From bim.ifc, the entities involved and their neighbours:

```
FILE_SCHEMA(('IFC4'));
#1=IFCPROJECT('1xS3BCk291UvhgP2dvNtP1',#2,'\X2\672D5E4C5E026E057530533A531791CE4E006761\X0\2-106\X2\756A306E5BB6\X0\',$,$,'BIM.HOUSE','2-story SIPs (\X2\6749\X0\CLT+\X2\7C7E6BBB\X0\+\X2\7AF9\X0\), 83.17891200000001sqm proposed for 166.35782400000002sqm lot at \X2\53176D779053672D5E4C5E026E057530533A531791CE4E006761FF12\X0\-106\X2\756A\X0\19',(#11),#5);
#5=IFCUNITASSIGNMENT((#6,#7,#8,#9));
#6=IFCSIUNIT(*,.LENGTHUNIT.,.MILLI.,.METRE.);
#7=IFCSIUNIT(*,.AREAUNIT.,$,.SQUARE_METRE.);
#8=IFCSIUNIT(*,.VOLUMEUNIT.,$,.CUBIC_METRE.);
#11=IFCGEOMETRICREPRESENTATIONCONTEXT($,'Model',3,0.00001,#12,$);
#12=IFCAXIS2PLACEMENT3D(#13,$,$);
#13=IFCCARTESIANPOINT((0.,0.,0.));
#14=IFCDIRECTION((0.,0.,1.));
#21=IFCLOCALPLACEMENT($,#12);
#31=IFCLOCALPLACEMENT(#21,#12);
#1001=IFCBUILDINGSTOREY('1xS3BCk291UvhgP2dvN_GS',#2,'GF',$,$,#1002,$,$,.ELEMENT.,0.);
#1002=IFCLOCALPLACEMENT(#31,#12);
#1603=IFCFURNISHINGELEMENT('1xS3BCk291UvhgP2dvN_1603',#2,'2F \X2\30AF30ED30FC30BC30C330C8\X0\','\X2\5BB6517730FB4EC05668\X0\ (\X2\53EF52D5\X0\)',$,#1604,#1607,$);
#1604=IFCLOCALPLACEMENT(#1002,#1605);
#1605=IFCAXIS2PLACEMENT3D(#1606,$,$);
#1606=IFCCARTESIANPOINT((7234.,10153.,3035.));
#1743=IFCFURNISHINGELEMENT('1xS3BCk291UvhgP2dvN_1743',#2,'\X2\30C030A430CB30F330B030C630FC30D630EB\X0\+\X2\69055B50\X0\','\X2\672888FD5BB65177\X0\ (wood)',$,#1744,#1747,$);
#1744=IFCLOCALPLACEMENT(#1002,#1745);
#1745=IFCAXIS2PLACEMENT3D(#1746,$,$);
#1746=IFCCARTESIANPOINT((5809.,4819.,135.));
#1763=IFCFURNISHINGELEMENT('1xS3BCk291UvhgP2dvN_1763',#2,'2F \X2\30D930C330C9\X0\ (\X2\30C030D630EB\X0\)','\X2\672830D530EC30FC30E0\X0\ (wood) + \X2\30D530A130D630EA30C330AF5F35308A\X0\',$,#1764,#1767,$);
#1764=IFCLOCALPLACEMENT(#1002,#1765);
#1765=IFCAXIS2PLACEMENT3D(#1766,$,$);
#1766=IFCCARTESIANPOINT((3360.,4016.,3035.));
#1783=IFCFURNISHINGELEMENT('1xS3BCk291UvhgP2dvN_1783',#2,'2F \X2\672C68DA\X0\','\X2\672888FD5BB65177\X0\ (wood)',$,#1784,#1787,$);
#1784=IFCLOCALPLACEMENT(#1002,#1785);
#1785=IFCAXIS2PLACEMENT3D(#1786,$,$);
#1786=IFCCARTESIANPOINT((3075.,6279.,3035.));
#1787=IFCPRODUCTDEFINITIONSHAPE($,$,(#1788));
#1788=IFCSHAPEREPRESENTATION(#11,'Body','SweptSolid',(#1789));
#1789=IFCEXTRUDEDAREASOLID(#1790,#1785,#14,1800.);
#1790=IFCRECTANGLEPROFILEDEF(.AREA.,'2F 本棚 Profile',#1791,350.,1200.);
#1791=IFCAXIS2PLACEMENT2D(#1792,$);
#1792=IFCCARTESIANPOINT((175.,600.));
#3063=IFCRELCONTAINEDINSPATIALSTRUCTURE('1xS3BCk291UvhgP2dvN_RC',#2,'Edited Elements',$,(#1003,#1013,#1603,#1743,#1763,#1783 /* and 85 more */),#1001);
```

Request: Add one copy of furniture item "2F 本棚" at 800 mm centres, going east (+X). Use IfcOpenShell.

```python
import numpy as np
import ifcopenshell
import ifcopenshell.api.geometry
import ifcopenshell.api.root
import ifcopenshell.util.element
import ifcopenshell.util.placement

model = ifcopenshell.open("bim.ifc")


def reuse_history(source, copy):
    """copy_class also copies each property set's owner history, people and application; keep the originals."""
    for rel in copy.IsDefinedBy:
        if rel.is_a("IfcRelDefinesByProperties") and (history := rel.RelatingPropertyDefinition.OwnerHistory):
            rel.RelatingPropertyDefinition.OwnerHistory = source.OwnerHistory
            ifcopenshell.util.element.remove_deep2(model, history)


source = model.by_guid("1xS3BCk291UvhgP2dvN_1783")
base = ifcopenshell.util.placement.get_local_placement(source.ObjectPlacement)
step = np.array([1.0, 0.0, 0.0]) * 800.0

for i in range(1, 2):
    copy = ifcopenshell.api.root.copy_class(model, product=source)
    copy.Representation = ifcopenshell.util.element.copy_deep(
        model, source.Representation, exclude=["IfcGeometricRepresentationContext", "IfcRepresentationMap"]
    )
    reuse_history(source, copy)
    matrix = base.copy()
    matrix[:3, 3] += i * step
    print("added at", matrix[:3, 3].round(3) + 0.0)
    ifcopenshell.api.geometry.edit_object_placement(model, product=copy, matrix=matrix, is_si=False)

model.write("bim_updated.ifc")
```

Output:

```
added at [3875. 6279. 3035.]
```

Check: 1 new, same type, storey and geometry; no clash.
